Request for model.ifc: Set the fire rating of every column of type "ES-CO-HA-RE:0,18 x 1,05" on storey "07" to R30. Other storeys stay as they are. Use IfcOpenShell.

First a look at what the model holds.

```python
import ifcopenshell
import ifcopenshell.util.element

model = ifcopenshell.open("model.ifc")
print(model.schema)
storey = next(s for s in model.by_type("IfcBuildingStorey") if s.Name == "07")
columns = [e for e in ifcopenshell.util.element.get_decomposition(storey) if e.is_a("IfcColumn")]
seen = {}
for e in columns:
    element_type = ifcopenshell.util.element.get_type(e)
    key = (element_type.Name if element_type != e and element_type else None, ifcopenshell.util.element.get_pset(e, "Pset_ColumnCommon", "FireRating"))
    seen[key] = seen.get(key, 0) + 1
for (name, value), count in sorted(seen.items(), key=str):
    print(count, "x", name, "|", value)
```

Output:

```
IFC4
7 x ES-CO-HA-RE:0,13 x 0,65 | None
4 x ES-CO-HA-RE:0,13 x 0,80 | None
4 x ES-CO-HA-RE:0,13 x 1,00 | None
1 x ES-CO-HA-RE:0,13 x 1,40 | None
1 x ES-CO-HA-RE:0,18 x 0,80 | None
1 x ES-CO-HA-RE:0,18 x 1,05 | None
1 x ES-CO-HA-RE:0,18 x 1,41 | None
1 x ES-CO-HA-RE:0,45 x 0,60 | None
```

```python
import ifcopenshell
import ifcopenshell.api.pset
import ifcopenshell.util.element

model = ifcopenshell.open("model.ifc")

storey = next(s for s in model.by_type("IfcBuildingStorey") if s.Name == "07")
columns = [e for e in ifcopenshell.util.element.get_decomposition(storey) if e.is_a("IfcColumn")]

count = 0
for e in columns:
    element_type = ifcopenshell.util.element.get_type(e)
    if element_type in (None, e) or element_type.Name != "ES-CO-HA-RE:0,18 x 1,05":
        continue
    # add_pset returns the element's existing set when there is one.
    pset = ifcopenshell.api.pset.add_pset(model, product=e, name="Pset_ColumnCommon")
    ifcopenshell.api.pset.edit_pset(model, pset=pset, properties={"FireRating": "R30"})
    count += 1

print(count, "columns updated")

model.write("model_rev.ifc")
```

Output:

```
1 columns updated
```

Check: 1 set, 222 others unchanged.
